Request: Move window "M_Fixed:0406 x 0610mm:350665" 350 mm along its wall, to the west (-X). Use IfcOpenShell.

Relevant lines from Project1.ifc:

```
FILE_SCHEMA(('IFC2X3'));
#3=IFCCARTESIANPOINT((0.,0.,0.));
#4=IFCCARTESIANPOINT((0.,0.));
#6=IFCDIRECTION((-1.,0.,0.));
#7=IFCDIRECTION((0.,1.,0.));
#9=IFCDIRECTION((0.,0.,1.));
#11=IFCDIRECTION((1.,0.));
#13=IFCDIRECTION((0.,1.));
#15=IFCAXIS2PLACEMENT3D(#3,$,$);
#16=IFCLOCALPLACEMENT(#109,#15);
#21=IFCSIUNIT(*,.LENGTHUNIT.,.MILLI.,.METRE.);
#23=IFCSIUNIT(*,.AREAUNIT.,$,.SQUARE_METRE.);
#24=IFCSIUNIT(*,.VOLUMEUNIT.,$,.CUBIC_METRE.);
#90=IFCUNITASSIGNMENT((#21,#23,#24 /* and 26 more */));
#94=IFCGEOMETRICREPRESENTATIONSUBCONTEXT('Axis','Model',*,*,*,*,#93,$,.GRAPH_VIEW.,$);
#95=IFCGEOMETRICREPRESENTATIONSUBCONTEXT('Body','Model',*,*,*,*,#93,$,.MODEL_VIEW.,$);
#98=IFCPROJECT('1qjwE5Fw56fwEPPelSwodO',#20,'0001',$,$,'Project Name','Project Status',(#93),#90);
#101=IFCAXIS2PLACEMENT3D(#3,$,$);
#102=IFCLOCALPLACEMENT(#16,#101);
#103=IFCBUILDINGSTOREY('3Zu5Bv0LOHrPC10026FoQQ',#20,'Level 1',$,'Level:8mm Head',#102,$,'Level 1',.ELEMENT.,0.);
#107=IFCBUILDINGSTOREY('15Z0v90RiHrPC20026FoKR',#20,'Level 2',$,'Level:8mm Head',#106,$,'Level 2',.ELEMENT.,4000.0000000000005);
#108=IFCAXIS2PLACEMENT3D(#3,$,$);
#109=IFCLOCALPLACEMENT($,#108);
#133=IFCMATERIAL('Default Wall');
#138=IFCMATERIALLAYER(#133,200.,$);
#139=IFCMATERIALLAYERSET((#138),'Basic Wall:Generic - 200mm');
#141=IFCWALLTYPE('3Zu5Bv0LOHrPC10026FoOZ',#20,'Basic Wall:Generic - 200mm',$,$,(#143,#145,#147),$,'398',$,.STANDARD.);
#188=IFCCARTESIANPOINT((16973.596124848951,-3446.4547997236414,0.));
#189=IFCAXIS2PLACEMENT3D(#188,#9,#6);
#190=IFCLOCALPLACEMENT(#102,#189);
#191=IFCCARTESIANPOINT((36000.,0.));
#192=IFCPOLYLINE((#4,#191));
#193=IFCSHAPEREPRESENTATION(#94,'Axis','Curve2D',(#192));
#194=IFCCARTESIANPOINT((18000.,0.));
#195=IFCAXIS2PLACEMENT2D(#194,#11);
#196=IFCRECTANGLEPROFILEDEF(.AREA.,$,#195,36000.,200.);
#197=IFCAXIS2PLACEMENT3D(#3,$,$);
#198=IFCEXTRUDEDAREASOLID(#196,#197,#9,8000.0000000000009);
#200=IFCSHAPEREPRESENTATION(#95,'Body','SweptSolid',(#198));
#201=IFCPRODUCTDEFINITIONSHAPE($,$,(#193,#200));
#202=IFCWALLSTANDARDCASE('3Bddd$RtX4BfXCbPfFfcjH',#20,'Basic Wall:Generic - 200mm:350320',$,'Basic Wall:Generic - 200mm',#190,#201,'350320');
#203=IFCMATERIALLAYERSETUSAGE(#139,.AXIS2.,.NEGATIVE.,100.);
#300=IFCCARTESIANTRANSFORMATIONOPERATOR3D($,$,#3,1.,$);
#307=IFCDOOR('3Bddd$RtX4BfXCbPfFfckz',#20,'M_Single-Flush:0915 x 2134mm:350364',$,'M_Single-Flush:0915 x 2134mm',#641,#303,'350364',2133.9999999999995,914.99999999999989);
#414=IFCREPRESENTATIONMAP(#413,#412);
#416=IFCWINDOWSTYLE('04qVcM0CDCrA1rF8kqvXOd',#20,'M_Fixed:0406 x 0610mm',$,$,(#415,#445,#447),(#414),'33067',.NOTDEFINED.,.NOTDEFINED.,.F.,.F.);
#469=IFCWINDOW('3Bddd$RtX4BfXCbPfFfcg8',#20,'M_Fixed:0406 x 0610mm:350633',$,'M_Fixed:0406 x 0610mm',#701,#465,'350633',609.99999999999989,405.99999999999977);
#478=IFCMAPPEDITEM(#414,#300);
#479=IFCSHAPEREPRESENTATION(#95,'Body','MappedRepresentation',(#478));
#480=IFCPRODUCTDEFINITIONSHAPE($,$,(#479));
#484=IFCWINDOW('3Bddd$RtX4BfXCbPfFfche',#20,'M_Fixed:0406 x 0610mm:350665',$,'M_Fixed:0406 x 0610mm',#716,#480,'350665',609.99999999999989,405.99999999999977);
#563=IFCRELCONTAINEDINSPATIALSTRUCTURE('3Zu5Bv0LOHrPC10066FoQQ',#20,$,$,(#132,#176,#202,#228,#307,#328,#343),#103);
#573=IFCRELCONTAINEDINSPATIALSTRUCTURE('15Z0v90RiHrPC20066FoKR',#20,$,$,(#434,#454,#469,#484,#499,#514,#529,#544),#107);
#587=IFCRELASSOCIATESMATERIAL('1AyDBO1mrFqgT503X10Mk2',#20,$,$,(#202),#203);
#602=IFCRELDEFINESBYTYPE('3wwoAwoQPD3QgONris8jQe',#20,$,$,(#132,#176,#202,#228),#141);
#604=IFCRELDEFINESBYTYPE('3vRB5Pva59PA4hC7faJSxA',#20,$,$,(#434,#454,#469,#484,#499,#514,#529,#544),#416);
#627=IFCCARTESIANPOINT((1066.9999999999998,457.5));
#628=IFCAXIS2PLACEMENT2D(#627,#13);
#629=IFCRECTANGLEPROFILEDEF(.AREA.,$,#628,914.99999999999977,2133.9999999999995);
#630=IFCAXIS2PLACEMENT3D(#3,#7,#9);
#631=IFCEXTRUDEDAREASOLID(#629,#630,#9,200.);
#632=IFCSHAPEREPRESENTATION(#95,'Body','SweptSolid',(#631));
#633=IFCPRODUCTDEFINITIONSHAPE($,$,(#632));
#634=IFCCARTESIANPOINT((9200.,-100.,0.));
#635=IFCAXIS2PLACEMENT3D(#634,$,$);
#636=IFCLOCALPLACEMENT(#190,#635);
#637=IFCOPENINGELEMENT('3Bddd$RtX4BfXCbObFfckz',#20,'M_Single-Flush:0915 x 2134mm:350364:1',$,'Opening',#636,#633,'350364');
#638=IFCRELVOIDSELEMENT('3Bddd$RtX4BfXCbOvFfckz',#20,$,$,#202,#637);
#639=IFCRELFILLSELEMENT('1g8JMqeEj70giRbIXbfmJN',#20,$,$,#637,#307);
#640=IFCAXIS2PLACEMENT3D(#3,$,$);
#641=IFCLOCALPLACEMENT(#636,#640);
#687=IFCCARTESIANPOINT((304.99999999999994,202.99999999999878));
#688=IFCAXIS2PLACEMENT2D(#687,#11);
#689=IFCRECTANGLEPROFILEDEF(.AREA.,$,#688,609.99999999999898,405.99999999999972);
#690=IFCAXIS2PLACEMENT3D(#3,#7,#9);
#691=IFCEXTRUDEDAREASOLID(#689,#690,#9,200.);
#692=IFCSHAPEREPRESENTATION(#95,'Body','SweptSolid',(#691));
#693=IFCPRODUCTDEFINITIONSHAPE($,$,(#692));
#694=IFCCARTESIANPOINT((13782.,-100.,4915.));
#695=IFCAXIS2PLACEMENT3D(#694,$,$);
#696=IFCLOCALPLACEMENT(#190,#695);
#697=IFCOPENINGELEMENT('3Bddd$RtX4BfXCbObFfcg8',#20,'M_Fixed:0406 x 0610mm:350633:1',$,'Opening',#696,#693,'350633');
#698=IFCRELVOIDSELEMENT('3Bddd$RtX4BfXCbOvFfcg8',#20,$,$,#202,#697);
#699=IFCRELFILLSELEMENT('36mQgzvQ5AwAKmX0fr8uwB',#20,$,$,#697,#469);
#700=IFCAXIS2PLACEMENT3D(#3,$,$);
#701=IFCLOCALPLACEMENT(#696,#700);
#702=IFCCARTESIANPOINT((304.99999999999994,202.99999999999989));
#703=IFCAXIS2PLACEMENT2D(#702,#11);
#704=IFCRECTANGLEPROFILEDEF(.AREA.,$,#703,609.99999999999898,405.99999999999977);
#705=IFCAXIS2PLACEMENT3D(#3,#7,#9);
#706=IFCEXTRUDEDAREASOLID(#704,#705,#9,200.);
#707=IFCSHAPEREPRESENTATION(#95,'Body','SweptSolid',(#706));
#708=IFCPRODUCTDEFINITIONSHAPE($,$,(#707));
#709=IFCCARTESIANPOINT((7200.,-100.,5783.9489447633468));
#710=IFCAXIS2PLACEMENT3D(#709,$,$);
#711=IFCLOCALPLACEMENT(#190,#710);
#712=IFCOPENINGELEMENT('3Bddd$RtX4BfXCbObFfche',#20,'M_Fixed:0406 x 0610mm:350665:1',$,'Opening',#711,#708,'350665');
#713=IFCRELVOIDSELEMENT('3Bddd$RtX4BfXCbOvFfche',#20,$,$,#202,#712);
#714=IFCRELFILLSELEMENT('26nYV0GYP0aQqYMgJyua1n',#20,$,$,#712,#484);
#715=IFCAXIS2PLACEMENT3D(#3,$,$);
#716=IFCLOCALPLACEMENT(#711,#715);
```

```python
import ifcopenshell
import ifcopenshell.api.geometry
import ifcopenshell.util.placement
import ifcopenshell.util.unit

model = ifcopenshell.open("Project1.ifc")
unit_scale = ifcopenshell.util.unit.calculate_unit_scale(model)

window = model.by_guid("3Bddd$RtX4BfXCbPfFfche")
opening = window.FillsVoids[0].RelatingOpeningElement
wall = opening.VoidsElements[0].RelatingBuildingElement

wall_matrix = ifcopenshell.util.placement.get_local_placement(wall.ObjectPlacement)
shift = wall_matrix[:3, 0] * 0.35 / unit_scale
before = ifcopenshell.util.placement.get_local_placement(window.ObjectPlacement)[:3, 3].copy()

# The window is placed relative to its opening, so it follows when the opening moves.
matrix = ifcopenshell.util.placement.get_local_placement(opening.ObjectPlacement)
matrix[:3, 3] += shift
ifcopenshell.api.geometry.edit_object_placement(
    model, product=opening, matrix=matrix, is_si=False, should_transform_children=True
)

after = ifcopenshell.util.placement.get_local_placement(window.ObjectPlacement)[:3, 3]
print("window moved by", (after - before).round(3) + 0.0)

model.write("Project1_v2.ifc")
```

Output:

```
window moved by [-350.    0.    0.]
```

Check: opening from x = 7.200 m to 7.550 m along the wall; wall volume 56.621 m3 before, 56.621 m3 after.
